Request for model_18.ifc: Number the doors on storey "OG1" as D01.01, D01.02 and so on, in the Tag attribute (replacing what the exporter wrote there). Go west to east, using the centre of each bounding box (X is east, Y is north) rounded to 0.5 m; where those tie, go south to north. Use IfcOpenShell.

First a look at what the model holds.

```python
import ifcopenshell
import ifcopenshell.util.element
import ifcopenshell.util.placement

model = ifcopenshell.open("model_18.ifc")
print(model.schema)
storey = next(s for s in model.by_type("IfcBuildingStorey") if s.Name == "OG1")
doors = [e for e in ifcopenshell.util.element.get_decomposition(storey) if e.is_a("IfcDoor")]
for e in sorted(doors, key=lambda e: e.id()):
    origin = ifcopenshell.util.placement.get_local_placement(e.ObjectPlacement)[:3, 3]
    print(e.id(), e.Tag, e.Name, origin.round(2) + 0.0, sep=" | ")
```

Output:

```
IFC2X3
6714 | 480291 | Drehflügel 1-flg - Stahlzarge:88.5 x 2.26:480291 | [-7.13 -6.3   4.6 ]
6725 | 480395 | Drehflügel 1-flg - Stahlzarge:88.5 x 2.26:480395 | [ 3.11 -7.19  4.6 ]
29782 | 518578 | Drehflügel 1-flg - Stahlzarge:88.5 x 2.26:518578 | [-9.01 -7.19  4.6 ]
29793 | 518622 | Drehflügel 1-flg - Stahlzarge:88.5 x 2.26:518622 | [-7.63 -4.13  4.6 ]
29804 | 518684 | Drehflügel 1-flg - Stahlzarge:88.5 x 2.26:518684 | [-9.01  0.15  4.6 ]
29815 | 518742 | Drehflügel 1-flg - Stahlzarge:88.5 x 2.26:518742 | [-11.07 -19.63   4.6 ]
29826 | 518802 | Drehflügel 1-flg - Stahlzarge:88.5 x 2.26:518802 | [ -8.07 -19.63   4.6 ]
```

```python
import ifcopenshell
import ifcopenshell.geom
import ifcopenshell.util.element
import ifcopenshell.util.shape

model = ifcopenshell.open("model_18.ifc")
settings = ifcopenshell.geom.settings()
settings.set("use-world-coords", True)


def centre(element):
    shape = ifcopenshell.geom.create_shape(settings, element)
    return ifcopenshell.util.shape.get_bbox_centroid(shape.geometry)


storey = next(s for s in model.by_type("IfcBuildingStorey") if s.Name == "OG1")
doors = [e for e in ifcopenshell.util.element.get_decomposition(storey) if e.is_a("IfcDoor")]

# Insertion points can sit at a corner or the storey origin, so sort by the geometry (in metres).
centres = {e: centre(e) for e in doors}
doors.sort(key=lambda e: (round(centres[e][0] / 0.5), centres[e][1]))

for i, e in enumerate(doors, start=1):
    number = f"D01.{i:02d}"
    e.Tag = number
    print(e.id(), number)

model.write("model_18_v2.ifc")
```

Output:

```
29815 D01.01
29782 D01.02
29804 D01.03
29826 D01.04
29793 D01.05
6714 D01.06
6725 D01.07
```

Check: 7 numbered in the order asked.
